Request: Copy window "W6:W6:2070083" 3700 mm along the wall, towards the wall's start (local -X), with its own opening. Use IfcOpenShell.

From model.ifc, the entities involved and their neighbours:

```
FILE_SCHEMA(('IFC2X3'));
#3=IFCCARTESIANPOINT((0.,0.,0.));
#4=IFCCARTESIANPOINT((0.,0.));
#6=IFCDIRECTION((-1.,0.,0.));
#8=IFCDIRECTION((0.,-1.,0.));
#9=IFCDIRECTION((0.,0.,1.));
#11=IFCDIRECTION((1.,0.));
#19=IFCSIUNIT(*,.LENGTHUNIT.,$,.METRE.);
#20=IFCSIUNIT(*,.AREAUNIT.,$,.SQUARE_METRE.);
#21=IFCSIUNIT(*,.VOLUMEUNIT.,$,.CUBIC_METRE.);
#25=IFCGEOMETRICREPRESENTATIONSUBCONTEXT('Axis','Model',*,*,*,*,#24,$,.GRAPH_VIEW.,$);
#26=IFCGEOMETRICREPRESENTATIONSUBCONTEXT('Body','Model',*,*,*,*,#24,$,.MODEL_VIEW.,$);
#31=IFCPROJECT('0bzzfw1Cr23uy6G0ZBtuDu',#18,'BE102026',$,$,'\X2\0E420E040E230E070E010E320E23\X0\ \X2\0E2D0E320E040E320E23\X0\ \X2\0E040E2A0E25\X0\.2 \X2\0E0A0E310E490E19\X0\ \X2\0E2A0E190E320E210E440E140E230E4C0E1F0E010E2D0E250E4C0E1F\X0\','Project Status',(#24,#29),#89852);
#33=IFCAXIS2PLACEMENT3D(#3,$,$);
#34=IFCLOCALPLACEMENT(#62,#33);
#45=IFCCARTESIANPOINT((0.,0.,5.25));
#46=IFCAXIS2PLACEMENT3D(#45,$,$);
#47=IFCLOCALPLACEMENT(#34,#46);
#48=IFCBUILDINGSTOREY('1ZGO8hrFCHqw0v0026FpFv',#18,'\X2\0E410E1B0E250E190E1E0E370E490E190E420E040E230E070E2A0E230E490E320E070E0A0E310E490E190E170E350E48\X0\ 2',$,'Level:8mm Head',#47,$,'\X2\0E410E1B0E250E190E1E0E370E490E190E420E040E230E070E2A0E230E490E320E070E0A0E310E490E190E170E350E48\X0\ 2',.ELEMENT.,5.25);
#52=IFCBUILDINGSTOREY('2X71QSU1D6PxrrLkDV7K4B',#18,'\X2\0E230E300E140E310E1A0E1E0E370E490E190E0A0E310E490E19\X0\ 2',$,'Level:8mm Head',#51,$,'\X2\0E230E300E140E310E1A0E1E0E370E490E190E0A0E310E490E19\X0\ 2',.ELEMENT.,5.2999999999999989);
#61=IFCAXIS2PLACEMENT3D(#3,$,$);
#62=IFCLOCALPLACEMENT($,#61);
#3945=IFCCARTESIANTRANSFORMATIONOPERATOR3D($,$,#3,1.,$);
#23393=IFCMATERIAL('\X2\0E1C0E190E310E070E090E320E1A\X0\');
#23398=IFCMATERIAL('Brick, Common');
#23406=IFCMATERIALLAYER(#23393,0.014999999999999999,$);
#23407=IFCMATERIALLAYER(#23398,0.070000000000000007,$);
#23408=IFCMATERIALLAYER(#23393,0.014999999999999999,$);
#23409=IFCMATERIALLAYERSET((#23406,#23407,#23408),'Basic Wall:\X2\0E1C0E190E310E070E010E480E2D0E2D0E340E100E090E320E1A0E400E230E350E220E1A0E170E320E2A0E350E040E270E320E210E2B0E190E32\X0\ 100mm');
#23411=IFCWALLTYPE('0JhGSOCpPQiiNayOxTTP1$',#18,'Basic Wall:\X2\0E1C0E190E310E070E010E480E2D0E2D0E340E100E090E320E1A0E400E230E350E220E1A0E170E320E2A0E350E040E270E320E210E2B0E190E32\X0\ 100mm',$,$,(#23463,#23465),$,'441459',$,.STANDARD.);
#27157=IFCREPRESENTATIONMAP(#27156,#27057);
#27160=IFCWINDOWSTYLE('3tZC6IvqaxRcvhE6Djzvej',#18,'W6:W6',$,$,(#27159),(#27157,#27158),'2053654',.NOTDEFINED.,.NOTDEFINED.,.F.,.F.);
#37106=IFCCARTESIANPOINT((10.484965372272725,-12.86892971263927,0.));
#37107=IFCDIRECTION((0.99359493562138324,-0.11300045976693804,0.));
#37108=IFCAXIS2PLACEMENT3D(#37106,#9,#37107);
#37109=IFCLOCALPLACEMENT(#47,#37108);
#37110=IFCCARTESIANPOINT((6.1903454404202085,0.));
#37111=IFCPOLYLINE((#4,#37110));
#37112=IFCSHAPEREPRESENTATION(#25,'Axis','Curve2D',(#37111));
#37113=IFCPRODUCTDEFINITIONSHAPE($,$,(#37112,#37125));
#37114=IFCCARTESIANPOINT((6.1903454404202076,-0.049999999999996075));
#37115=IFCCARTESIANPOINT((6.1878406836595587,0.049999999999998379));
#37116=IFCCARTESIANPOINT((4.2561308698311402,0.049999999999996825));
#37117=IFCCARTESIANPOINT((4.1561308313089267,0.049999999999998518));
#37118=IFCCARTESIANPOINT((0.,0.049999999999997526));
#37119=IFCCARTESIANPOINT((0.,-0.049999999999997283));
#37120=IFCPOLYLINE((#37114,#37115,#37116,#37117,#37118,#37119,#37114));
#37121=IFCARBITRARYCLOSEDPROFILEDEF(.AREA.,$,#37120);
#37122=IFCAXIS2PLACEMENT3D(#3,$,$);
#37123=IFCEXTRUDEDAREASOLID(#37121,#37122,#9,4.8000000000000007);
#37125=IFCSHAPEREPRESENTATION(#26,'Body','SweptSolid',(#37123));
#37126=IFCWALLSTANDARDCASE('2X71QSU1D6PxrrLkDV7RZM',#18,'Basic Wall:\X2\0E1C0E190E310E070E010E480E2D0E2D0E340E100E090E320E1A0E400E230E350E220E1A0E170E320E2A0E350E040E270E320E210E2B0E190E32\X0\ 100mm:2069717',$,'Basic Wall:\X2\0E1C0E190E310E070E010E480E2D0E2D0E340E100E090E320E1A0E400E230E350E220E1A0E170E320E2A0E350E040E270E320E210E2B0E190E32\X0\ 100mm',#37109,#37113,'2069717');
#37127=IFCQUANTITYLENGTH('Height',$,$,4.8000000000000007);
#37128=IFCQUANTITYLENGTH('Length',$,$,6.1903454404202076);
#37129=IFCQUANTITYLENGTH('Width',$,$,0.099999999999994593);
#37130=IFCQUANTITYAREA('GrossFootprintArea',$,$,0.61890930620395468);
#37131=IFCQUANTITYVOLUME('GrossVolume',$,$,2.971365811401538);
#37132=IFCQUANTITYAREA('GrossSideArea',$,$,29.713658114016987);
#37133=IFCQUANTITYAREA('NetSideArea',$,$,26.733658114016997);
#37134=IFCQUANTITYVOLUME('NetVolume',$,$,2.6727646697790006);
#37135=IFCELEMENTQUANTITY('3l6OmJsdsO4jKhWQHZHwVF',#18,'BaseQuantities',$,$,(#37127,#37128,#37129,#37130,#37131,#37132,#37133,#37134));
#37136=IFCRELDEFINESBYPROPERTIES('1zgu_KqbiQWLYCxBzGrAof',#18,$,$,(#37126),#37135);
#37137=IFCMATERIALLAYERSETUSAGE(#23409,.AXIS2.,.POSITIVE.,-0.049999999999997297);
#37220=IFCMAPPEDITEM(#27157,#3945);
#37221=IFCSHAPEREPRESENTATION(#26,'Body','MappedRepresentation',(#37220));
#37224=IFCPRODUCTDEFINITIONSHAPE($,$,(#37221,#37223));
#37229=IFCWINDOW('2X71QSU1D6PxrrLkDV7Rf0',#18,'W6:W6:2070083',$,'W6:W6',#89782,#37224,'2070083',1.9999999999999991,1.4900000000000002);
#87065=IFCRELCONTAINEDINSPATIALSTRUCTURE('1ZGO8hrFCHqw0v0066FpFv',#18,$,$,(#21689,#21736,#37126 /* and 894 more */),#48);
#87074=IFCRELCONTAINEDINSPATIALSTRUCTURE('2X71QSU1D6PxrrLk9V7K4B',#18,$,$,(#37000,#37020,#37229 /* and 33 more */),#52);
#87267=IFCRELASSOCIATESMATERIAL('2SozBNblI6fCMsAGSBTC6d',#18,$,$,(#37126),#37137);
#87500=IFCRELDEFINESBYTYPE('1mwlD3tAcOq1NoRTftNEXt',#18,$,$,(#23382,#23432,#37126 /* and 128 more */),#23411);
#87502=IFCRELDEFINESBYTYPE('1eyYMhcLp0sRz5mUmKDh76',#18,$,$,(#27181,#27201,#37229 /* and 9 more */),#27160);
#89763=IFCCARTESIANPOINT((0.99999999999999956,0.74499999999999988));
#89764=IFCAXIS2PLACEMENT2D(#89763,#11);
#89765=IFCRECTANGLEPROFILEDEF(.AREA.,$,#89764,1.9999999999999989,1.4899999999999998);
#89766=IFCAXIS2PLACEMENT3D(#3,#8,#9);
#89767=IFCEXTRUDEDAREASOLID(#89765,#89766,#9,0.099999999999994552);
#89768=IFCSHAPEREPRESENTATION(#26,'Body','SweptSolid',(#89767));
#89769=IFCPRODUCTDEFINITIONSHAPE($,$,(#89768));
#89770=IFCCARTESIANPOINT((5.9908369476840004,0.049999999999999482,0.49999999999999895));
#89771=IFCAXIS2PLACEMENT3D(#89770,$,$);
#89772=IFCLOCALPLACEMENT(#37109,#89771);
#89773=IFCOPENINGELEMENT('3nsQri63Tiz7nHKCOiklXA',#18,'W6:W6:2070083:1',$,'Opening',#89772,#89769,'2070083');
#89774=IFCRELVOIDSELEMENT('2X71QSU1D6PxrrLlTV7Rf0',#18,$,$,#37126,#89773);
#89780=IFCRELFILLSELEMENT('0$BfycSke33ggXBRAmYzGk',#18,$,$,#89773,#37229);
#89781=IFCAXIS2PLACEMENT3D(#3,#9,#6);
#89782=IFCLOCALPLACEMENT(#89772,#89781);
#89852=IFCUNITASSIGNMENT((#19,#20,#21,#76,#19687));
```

```python
import ifcopenshell
import ifcopenshell.api.feature
import ifcopenshell.api.geometry
import ifcopenshell.api.pset
import ifcopenshell.api.root
import ifcopenshell.geom
import ifcopenshell.util.element
import ifcopenshell.util.placement
import ifcopenshell.util.shape
import ifcopenshell.util.unit

model = ifcopenshell.open("model.ifc")
unit_scale = ifcopenshell.util.unit.calculate_unit_scale(model)
area_scale = ifcopenshell.util.unit.calculate_unit_scale(model, "AREAUNIT")
volume_scale = ifcopenshell.util.unit.calculate_unit_scale(model, "VOLUMEUNIT")
settings = ifcopenshell.geom.settings()


def volume(element):
    """Net volume in cubic metres, openings subtracted."""
    shape = ifcopenshell.geom.create_shape(settings, element)
    return ifcopenshell.util.shape.get_volume(shape.geometry)


def reuse_history(source, copy):
    """copy_class also copies each property set's owner history, people and application; keep the originals."""
    for rel in copy.IsDefinedBy:
        if rel.is_a("IfcRelDefinesByProperties") and (history := rel.RelatingPropertyDefinition.OwnerHistory):
            rel.RelatingPropertyDefinition.OwnerHistory = source.OwnerHistory
            ifcopenshell.util.element.remove_deep2(model, history)


window = model.by_guid("2X71QSU1D6PxrrLkDV7Rf0")
opening = window.FillsVoids[0].RelatingOpeningElement
wall = opening.VoidsElements[0].RelatingBuildingElement
before = volume(wall)
shift = ifcopenshell.util.placement.get_local_placement(wall.ObjectPlacement)[:3, 0] * -3.7 / unit_scale

# copy_class copies the void relationship, type, container and properties, but no geometry.
new_opening = ifcopenshell.api.root.copy_class(model, product=opening)
new_opening.Representation = ifcopenshell.util.element.copy_deep(
    model, opening.Representation, exclude=["IfcGeometricRepresentationContext", "IfcRepresentationMap"]
)
new_opening.Name = "W6:W6"
new_opening.Tag = None
reuse_history(opening, new_opening)
new_window = ifcopenshell.api.root.copy_class(model, product=window)
new_window.Representation = ifcopenshell.util.element.copy_deep(
    model, window.Representation, exclude=["IfcGeometricRepresentationContext", "IfcRepresentationMap"]
)
new_window.Name = "W6:W6"
new_window.Tag = None
reuse_history(window, new_window)
fills = ifcopenshell.api.feature.add_filling(model, opening=new_opening, element=new_window)
fills.OwnerHistory = new_window.OwnerHistory  # required in IFC2X3

for old, new in ((opening, new_opening), (window, new_window)):
    matrix = ifcopenshell.util.placement.get_local_placement(old.ObjectPlacement)
    matrix[:3, 3] += shift
    ifcopenshell.api.geometry.edit_object_placement(model, product=new, matrix=matrix, is_si=False)

after = volume(wall)
thickness = 0.1  # wall thickness in metres

# Update the wall's stored quantities.
qto = model.by_id(ifcopenshell.util.element.get_pset(wall, "BaseQuantities", should_inherit=False)["id"])
ifcopenshell.api.pset.edit_qto(model, qto=qto, properties={
    "NetSideArea": after / thickness / area_scale,
    "NetVolume": after / volume_scale,
})

print(f"wall volume {before:.3f} -> {after:.3f} m3")

model.write("model_updated.ifc")
```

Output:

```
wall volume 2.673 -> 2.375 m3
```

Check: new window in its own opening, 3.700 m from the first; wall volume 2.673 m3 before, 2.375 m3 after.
